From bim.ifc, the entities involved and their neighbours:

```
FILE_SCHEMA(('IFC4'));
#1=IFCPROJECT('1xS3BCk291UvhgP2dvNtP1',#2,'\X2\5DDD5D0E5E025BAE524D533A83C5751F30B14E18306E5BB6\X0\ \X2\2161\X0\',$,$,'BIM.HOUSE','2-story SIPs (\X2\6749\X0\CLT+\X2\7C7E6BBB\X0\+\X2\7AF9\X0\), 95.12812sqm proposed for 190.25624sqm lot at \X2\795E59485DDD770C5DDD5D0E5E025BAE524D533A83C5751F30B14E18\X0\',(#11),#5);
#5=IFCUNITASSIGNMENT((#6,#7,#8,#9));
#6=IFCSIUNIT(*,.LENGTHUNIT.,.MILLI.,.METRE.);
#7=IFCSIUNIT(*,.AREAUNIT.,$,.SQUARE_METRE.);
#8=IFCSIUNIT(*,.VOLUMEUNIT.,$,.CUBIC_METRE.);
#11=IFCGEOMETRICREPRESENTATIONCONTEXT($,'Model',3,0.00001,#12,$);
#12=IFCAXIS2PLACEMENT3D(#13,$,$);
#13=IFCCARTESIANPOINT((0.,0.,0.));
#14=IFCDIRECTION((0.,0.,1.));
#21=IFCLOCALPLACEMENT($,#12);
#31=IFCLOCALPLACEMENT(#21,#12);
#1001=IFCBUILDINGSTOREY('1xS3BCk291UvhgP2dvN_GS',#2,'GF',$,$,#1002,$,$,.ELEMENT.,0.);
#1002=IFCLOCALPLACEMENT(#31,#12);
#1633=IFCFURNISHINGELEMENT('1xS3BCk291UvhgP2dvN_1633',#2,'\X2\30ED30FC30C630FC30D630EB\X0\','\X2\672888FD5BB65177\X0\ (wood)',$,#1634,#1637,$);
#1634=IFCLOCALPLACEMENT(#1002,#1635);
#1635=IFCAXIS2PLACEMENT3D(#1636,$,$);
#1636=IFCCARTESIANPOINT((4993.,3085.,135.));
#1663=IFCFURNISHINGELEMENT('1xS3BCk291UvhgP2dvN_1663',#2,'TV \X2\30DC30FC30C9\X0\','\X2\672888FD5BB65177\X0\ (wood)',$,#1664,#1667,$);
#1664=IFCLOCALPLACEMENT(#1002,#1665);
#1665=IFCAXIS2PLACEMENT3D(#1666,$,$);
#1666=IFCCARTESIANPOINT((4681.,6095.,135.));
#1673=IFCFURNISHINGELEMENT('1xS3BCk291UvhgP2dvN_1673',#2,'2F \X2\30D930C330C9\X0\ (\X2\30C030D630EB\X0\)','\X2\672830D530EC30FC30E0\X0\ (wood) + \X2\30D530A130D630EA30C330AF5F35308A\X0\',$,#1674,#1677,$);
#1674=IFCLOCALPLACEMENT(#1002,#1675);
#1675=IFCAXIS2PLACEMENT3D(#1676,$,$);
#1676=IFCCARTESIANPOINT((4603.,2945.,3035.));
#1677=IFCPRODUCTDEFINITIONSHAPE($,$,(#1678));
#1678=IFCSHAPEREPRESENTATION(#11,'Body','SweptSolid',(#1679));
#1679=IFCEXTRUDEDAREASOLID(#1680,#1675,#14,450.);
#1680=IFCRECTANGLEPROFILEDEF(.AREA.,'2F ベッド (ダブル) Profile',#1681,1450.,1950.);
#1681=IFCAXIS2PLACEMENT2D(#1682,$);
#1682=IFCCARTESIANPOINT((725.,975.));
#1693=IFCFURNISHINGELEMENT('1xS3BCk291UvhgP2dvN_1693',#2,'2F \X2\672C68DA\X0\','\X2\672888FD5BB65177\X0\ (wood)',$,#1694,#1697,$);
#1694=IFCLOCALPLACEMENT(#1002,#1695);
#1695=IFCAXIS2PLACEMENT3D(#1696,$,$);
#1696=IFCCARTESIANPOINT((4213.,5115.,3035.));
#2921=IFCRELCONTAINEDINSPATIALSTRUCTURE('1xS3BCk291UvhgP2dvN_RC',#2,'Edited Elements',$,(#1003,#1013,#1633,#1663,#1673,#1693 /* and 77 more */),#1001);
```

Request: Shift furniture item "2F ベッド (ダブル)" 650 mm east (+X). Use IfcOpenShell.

```python
import ifcopenshell
import ifcopenshell.api.geometry
import ifcopenshell.util.placement
import ifcopenshell.util.unit

model = ifcopenshell.open("bim.ifc")
unit_scale = ifcopenshell.util.unit.calculate_unit_scale(model)

item = model.by_guid("1xS3BCk291UvhgP2dvN_1673")
matrix = ifcopenshell.util.placement.get_local_placement(item.ObjectPlacement)
matrix[0, 3] += 0.65 / unit_scale
ifcopenshell.api.geometry.edit_object_placement(model, product=item, matrix=matrix, is_si=False)

print(ifcopenshell.util.placement.get_local_placement(item.ObjectPlacement).round(3) + 0.0)

model.write("bim_v2.ifc")
```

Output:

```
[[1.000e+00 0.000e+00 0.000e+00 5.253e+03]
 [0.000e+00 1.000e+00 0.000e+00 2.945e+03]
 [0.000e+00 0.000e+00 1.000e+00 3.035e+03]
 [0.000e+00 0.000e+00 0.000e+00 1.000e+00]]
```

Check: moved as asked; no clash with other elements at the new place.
